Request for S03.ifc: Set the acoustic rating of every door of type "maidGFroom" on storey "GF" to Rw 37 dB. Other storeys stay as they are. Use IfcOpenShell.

First a look at what the model holds.

```python
import ifcopenshell
import ifcopenshell.util.element

model = ifcopenshell.open("S03.ifc")
print(model.schema)
storey = next(s for s in model.by_type("IfcBuildingStorey") if s.Name == "GF")
doors = [e for e in ifcopenshell.util.element.get_decomposition(storey) if e.is_a("IfcDoor")]
seen = {}
for e in doors:
    element_type = ifcopenshell.util.element.get_type(e)
    key = (element_type.Name if element_type != e and element_type else None, ifcopenshell.util.element.get_pset(e, "Pset_DoorCommon", "AcousticRating"))
    seen[key] = seen.get(key, 0) + 1
for (name, value), count in sorted(seen.items(), key=str):
    print(count, "x", name, "|", value)
```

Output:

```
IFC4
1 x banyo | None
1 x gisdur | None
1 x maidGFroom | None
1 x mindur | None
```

```python
import ifcopenshell
import ifcopenshell.api.pset
import ifcopenshell.util.element

model = ifcopenshell.open("S03.ifc")

storey = next(s for s in model.by_type("IfcBuildingStorey") if s.Name == "GF")
doors = [e for e in ifcopenshell.util.element.get_decomposition(storey) if e.is_a("IfcDoor")]

count = 0
for e in doors:
    element_type = ifcopenshell.util.element.get_type(e)
    if element_type in (None, e) or element_type.Name != "maidGFroom":
        continue
    # add_pset returns the element's existing set when there is one.
    pset = ifcopenshell.api.pset.add_pset(model, product=e, name="Pset_DoorCommon")
    ifcopenshell.api.pset.edit_pset(model, pset=pset, properties={"AcousticRating": "Rw 37 dB"})
    count += 1

print(count, "doors updated")

model.write("S03_updated.ifc")
```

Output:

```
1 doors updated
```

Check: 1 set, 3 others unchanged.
